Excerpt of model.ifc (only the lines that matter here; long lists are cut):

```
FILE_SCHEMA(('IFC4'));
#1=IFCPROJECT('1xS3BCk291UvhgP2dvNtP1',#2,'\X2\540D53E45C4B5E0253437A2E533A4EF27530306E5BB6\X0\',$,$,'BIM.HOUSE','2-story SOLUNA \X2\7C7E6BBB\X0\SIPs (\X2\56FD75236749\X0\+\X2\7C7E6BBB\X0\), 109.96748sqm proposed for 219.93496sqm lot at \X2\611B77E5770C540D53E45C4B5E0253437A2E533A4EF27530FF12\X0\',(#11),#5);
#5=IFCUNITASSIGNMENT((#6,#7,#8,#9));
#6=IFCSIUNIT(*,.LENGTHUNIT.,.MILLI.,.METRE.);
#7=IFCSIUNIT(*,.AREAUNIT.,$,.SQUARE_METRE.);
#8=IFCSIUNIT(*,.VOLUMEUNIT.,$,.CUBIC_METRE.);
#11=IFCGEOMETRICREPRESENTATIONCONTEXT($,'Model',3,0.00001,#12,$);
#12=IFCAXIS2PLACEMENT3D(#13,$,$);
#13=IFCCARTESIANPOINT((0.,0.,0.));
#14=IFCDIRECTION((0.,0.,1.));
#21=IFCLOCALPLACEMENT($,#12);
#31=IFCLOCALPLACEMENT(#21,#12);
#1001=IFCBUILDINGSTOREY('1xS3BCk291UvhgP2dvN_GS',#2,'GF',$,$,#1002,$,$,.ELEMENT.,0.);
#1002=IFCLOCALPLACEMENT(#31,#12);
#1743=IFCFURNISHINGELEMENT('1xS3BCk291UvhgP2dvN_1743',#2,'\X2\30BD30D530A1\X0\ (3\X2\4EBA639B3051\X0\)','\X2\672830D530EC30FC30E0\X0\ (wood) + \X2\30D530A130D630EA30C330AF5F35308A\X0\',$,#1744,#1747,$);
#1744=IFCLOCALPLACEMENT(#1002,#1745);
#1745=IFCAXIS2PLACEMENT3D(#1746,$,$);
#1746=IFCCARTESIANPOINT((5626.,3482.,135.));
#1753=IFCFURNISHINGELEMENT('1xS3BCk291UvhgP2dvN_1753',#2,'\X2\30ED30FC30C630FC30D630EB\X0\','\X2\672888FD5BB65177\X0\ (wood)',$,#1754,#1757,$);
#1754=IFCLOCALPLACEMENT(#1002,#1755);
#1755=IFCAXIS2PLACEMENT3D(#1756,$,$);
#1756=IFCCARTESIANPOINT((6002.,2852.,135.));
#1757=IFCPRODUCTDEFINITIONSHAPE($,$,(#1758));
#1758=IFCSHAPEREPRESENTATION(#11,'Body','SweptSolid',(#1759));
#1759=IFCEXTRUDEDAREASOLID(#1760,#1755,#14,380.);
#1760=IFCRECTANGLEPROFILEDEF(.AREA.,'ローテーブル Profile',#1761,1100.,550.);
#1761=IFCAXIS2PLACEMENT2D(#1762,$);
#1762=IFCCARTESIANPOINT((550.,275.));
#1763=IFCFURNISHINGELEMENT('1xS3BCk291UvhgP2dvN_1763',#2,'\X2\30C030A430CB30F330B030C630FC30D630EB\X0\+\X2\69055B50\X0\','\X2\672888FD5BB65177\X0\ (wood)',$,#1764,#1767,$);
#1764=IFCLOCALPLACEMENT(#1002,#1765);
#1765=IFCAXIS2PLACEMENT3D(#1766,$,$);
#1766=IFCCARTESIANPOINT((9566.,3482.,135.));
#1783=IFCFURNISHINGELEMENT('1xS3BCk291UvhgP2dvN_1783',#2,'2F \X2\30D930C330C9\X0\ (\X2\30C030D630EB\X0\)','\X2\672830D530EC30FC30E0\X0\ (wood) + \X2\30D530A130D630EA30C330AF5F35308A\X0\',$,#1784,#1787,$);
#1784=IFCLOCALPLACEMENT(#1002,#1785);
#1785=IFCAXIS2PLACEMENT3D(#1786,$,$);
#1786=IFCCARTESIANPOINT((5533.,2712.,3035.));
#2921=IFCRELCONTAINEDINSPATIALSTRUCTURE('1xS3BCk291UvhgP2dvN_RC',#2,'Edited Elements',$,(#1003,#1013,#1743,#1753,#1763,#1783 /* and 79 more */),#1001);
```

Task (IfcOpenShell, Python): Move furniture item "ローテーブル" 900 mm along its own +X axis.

```python
import ifcopenshell
import ifcopenshell.api.geometry
import ifcopenshell.util.placement
import ifcopenshell.util.unit

model = ifcopenshell.open("model.ifc")
unit_scale = ifcopenshell.util.unit.calculate_unit_scale(model)

item = model.by_guid("1xS3BCk291UvhgP2dvN_1753")
matrix = ifcopenshell.util.placement.get_local_placement(item.ObjectPlacement)
matrix[:3, 3] += matrix[:3, 0] * 0.9 / unit_scale
ifcopenshell.api.geometry.edit_object_placement(model, product=item, matrix=matrix, is_si=False)

print(ifcopenshell.util.placement.get_local_placement(item.ObjectPlacement).round(3) + 0.0)

model.write("model_edited.ifc")
```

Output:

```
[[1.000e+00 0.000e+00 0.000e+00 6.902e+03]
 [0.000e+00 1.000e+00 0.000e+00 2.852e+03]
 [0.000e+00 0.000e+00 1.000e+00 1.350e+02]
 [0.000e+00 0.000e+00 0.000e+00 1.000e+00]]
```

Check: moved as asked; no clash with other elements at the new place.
